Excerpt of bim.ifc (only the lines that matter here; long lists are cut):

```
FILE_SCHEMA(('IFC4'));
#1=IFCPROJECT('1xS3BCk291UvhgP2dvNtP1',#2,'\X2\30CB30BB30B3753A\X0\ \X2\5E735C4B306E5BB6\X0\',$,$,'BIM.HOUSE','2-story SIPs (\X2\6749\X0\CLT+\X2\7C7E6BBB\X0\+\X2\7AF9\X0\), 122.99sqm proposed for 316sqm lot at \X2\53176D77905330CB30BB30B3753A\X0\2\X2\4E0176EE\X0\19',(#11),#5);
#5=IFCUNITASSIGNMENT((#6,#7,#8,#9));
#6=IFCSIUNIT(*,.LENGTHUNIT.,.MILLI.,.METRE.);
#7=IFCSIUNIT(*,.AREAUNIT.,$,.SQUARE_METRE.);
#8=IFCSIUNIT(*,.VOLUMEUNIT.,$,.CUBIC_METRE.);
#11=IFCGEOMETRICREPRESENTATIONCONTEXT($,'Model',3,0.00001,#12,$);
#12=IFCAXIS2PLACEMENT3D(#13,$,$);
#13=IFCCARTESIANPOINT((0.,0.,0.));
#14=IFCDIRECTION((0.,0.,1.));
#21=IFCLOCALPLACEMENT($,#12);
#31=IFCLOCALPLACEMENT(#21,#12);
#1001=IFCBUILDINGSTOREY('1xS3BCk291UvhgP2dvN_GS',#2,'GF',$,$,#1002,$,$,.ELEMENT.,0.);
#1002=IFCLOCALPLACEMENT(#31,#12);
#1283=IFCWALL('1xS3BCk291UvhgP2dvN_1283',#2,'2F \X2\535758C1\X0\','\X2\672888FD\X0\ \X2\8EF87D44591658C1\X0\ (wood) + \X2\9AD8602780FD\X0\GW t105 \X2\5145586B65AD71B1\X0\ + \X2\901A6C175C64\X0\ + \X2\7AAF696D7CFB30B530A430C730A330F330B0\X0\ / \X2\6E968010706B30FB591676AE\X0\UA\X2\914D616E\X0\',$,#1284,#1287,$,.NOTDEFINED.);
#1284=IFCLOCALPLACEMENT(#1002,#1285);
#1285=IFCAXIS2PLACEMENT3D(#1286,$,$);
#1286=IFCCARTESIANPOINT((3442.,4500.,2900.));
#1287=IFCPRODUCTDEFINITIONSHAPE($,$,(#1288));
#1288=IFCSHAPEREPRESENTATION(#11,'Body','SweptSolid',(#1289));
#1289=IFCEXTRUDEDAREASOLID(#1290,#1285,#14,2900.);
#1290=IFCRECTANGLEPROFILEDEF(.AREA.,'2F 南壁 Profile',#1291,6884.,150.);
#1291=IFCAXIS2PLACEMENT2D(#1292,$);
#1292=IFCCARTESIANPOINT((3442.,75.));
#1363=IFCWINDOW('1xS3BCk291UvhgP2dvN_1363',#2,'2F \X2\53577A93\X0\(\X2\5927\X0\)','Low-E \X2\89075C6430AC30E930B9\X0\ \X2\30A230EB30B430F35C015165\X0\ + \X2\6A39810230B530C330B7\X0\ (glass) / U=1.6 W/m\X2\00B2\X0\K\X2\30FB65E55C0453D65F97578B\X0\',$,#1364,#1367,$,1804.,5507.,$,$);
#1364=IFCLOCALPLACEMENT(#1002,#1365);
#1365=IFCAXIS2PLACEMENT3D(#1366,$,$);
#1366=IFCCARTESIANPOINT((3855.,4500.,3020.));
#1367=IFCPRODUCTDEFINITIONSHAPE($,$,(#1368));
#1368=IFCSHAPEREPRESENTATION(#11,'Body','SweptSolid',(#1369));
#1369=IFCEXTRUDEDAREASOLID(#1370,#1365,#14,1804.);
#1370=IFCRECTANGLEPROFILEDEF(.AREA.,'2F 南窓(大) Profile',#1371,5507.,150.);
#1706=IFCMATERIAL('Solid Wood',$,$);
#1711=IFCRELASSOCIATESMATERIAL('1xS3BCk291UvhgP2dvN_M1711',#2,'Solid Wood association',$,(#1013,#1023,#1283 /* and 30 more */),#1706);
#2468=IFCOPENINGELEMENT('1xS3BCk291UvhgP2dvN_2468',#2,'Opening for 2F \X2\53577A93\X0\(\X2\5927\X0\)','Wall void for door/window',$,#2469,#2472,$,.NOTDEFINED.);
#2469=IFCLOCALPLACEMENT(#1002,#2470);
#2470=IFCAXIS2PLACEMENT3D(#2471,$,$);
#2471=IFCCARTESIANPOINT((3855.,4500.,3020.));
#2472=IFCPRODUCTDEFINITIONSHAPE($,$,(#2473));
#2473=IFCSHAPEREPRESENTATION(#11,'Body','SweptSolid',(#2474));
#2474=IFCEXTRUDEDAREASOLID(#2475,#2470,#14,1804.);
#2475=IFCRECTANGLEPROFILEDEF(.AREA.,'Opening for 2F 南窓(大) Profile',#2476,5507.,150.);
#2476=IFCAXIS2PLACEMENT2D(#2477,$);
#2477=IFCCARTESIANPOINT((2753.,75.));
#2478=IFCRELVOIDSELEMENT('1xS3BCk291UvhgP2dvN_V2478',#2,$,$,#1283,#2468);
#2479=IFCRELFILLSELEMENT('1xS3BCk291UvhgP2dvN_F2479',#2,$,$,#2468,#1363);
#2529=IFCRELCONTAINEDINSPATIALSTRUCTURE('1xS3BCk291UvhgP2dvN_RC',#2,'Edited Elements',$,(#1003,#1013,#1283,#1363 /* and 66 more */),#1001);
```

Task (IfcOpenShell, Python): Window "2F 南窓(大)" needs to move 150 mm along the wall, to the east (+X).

```python
import ifcopenshell
import ifcopenshell.api.geometry
import ifcopenshell.util.placement

model = ifcopenshell.open("bim.ifc")

window = model.by_guid("1xS3BCk291UvhgP2dvN_1363")
opening = window.FillsVoids[0].RelatingOpeningElement
wall = opening.VoidsElements[0].RelatingBuildingElement

wall_matrix = ifcopenshell.util.placement.get_local_placement(wall.ObjectPlacement)
shift = wall_matrix[:3, 0] * 150.0
before = ifcopenshell.util.placement.get_local_placement(window.ObjectPlacement)[:3, 3].copy()

# The window is not placed relative to its opening, so move both.
for product in (opening, window):
    matrix = ifcopenshell.util.placement.get_local_placement(product.ObjectPlacement)
    matrix[:3, 3] += shift
    ifcopenshell.api.geometry.edit_object_placement(model, product=product, matrix=matrix, is_si=False)

after = ifcopenshell.util.placement.get_local_placement(window.ObjectPlacement)[:3, 3]
print("window moved by", (after - before).round(3) + 0.0)

model.write("bim_rev.ifc")
```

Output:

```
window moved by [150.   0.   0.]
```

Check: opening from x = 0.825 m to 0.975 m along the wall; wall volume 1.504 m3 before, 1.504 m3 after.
